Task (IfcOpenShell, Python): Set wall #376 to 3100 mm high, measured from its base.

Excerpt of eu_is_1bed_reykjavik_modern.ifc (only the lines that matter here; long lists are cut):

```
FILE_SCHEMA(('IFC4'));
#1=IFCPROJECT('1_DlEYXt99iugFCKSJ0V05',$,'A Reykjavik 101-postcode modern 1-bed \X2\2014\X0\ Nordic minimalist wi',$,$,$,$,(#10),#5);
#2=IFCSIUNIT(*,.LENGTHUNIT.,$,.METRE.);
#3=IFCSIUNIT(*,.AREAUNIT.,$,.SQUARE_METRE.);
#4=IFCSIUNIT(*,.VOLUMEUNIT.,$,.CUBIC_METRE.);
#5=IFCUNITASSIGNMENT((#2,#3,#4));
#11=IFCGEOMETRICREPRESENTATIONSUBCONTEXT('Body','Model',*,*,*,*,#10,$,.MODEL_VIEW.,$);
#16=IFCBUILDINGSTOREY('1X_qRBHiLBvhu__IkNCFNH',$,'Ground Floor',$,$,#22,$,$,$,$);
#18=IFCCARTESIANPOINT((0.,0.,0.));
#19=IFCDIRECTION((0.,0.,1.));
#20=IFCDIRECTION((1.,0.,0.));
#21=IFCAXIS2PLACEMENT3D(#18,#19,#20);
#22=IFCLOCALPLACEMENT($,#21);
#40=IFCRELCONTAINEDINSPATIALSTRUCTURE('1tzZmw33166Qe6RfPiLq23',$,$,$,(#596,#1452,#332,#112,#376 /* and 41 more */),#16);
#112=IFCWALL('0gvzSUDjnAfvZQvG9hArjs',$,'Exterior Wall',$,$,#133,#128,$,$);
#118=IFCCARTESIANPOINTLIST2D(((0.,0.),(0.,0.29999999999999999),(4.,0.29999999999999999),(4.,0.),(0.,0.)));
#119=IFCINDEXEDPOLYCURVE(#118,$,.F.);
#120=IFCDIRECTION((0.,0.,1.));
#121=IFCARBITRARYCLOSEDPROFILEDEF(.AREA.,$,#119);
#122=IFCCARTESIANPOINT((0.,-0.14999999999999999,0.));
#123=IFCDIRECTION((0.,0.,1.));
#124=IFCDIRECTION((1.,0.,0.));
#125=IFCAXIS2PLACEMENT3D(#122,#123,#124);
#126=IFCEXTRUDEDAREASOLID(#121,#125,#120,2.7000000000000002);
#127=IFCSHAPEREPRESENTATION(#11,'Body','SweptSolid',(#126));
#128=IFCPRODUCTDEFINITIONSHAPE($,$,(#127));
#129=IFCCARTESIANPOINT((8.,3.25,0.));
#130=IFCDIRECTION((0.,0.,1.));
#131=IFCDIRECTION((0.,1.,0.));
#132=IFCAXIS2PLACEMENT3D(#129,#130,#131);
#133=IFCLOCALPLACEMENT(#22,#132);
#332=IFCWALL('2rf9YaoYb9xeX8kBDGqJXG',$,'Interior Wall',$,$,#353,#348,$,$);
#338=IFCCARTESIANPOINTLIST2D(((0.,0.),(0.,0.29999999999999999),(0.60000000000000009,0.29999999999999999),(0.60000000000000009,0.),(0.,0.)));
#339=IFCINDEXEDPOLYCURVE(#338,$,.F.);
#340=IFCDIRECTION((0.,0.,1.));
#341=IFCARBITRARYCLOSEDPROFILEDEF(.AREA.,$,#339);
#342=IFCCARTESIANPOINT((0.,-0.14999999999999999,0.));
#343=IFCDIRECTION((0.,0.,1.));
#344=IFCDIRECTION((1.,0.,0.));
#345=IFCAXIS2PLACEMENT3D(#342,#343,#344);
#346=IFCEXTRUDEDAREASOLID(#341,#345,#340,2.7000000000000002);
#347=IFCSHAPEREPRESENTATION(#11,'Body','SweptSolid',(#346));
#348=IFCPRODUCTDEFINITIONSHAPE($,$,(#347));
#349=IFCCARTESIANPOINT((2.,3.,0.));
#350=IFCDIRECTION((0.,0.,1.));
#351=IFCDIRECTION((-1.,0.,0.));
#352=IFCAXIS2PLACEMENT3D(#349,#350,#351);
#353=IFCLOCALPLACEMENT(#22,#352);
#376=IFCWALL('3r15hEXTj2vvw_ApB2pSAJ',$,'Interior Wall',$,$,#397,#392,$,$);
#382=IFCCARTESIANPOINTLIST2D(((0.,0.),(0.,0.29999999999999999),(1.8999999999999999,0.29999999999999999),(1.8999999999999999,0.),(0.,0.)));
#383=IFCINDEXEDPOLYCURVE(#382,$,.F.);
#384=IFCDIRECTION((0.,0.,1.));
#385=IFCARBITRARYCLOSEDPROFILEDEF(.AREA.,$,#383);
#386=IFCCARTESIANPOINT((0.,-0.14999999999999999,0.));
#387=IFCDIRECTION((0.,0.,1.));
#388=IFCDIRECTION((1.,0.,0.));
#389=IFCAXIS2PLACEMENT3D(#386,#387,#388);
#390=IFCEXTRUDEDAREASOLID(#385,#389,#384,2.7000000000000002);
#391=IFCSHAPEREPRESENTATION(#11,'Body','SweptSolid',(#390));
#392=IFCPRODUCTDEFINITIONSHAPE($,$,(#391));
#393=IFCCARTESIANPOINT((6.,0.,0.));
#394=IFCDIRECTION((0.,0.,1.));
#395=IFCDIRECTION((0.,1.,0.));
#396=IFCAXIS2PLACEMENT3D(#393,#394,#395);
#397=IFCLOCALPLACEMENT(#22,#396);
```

```python
import ifcopenshell
import ifcopenshell.geom
import ifcopenshell.util.representation
import ifcopenshell.util.shape
import ifcopenshell.util.unit

model = ifcopenshell.open("eu_is_1bed_reykjavik_modern.ifc")
unit_scale = ifcopenshell.util.unit.calculate_unit_scale(model)
settings = ifcopenshell.geom.settings()


def volume(element):
    """Net volume in cubic metres, openings subtracted."""
    shape = ifcopenshell.geom.create_shape(settings, element)
    return ifcopenshell.util.shape.get_volume(shape.geometry)


wall = model.by_guid("3r15hEXTj2vvw_ApB2pSAJ")
before = volume(wall)

body = ifcopenshell.util.representation.get_representation(wall, "Model", "Body")
solid = body.Items[0]
old_height = solid.Depth
solid.Depth = 3.1 / unit_scale
after = volume(wall)

print(f"height {old_height:g} -> {solid.Depth:g}, volume {before:.3f} -> {after:.3f} m3")

model.write("eu_is_1bed_reykjavik_modern-out.ifc")
```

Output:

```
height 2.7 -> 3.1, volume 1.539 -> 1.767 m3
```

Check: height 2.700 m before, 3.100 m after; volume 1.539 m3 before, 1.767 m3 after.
